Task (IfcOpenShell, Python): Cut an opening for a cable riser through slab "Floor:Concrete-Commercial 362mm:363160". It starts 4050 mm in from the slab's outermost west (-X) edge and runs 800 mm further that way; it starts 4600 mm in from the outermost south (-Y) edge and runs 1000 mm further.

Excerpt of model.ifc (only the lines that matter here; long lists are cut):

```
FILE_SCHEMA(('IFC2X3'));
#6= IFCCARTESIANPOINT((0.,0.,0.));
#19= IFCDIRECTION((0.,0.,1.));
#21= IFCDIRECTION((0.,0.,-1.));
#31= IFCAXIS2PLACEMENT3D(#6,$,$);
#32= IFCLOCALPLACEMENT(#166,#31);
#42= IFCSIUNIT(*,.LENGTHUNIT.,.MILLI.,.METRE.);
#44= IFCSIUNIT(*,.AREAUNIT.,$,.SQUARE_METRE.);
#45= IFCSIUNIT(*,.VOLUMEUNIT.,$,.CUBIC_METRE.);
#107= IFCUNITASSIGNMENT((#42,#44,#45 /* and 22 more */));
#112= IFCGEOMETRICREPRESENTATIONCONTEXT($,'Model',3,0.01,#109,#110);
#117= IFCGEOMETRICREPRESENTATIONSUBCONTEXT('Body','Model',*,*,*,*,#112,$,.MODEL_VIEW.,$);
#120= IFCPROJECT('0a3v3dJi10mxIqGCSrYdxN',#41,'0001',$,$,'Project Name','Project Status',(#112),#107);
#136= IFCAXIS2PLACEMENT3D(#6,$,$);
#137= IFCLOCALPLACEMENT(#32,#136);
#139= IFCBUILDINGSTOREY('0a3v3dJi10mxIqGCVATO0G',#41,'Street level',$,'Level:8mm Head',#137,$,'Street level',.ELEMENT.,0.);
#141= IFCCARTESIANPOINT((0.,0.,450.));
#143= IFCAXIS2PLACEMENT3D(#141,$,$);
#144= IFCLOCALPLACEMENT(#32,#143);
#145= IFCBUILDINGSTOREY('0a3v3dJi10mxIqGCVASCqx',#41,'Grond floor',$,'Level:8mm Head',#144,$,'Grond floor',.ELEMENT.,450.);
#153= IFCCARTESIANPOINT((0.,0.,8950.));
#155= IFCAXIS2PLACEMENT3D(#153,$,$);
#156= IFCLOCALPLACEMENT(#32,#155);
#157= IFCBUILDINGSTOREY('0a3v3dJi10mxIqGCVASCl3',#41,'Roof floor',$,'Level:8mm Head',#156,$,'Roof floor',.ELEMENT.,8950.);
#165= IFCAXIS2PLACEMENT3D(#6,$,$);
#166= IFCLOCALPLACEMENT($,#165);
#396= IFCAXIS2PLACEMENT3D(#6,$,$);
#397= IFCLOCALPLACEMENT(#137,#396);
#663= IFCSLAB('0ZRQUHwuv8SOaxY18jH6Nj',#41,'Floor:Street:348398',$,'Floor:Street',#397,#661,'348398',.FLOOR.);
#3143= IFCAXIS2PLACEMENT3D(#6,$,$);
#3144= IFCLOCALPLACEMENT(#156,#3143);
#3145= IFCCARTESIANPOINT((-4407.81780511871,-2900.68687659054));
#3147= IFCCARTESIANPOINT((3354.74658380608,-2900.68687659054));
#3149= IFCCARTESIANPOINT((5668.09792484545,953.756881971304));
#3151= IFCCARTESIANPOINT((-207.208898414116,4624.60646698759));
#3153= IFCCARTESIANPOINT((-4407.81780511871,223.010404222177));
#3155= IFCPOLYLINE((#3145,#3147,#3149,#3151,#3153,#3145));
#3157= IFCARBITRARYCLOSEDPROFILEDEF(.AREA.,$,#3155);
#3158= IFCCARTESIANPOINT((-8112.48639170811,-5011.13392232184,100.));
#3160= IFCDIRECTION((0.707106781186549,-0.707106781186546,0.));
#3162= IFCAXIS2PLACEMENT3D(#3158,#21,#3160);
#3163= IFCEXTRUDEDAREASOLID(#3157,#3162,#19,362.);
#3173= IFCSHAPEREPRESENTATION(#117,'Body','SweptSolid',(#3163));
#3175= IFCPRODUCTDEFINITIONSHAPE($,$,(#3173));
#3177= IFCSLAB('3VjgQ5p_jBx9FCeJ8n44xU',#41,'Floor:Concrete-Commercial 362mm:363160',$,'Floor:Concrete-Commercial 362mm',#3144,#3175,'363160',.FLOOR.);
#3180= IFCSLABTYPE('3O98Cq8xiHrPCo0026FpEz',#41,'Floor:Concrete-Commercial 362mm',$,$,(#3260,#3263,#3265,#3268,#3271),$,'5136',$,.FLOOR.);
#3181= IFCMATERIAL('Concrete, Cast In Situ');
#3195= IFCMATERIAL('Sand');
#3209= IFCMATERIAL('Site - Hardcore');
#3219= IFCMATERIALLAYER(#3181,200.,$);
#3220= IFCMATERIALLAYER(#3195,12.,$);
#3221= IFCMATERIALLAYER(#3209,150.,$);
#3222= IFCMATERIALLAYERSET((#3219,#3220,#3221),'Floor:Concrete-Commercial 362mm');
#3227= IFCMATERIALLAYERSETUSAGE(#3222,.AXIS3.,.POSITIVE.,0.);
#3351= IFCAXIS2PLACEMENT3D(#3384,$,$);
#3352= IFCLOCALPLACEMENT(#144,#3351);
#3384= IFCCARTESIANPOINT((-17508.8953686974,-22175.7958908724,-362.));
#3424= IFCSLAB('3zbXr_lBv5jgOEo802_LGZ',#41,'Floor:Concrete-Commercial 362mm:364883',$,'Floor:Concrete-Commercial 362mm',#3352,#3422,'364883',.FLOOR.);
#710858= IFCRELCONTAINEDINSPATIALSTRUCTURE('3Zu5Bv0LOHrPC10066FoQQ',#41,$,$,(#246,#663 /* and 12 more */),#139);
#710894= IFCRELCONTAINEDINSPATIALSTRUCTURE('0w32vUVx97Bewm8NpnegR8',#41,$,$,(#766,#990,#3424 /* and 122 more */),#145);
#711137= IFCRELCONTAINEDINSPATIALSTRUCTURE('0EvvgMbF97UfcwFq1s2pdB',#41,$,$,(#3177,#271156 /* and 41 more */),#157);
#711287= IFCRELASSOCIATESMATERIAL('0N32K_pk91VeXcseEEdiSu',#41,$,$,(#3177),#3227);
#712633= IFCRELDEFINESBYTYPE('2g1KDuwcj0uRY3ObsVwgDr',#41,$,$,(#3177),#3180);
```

```python
import numpy as np
import ifcopenshell
import ifcopenshell.api.feature
import ifcopenshell.api.geometry
import ifcopenshell.api.root
import ifcopenshell.geom
import ifcopenshell.util.placement
import ifcopenshell.util.representation
import ifcopenshell.util.shape
import ifcopenshell.util.unit

model = ifcopenshell.open("model.ifc")
unit_scale = ifcopenshell.util.unit.calculate_unit_scale(model)
settings = ifcopenshell.geom.settings()


def volume(element):
    """Net volume in cubic metres, openings subtracted."""
    shape = ifcopenshell.geom.create_shape(settings, element)
    return ifcopenshell.util.shape.get_volume(shape.geometry)


slab = model.by_guid("3VjgQ5p_jBx9FCeJ8n44xU")
before = volume(slab)

# Extent in the slab's own axes, in metres. The edges named are its -X and -Y sides.
slab_shape = ifcopenshell.geom.create_shape(settings, slab)
vertices = ifcopenshell.util.shape.get_vertices(slab_shape.geometry)
x_min, y_min, bottom = vertices.min(axis=0)
top = vertices[:, 2].max()

opening = ifcopenshell.api.root.create_entity(model, ifc_class="IfcOpeningElement", name="Cable riser opening")
context = ifcopenshell.util.representation.get_context(model, "Model", "Body", "MODEL_VIEW")
width, depth = 0.8, 1
outline = [(0.0, 0.0), (width, 0.0), (width, depth), (0.0, depth), (0.0, 0.0)]
# Overshoot both faces by 50 mm so the cut is clean.
shape = ifcopenshell.api.geometry.add_slab_representation(
    model, context=context, depth=top - bottom + 0.1, polyline=outline
)
ifcopenshell.api.geometry.assign_representation(model, product=opening, representation=shape)

matrix = ifcopenshell.util.placement.get_local_placement(slab.ObjectPlacement)
matrix[:, 3] = matrix @ np.append(np.array([x_min + 4.05, y_min + 4.6, bottom - 0.05]) / unit_scale, 1.0)
ifcopenshell.api.geometry.edit_object_placement(model, product=opening, matrix=matrix, is_si=False)
ifcopenshell.api.feature.add_feature(model, feature=opening, element=slab)

after = volume(slab)

print(f"slab volume {before:.3f} -> {after:.3f} m3")

model.write("model_updated.ifc")
```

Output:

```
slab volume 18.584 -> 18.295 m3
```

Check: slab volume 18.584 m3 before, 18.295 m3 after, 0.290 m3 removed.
